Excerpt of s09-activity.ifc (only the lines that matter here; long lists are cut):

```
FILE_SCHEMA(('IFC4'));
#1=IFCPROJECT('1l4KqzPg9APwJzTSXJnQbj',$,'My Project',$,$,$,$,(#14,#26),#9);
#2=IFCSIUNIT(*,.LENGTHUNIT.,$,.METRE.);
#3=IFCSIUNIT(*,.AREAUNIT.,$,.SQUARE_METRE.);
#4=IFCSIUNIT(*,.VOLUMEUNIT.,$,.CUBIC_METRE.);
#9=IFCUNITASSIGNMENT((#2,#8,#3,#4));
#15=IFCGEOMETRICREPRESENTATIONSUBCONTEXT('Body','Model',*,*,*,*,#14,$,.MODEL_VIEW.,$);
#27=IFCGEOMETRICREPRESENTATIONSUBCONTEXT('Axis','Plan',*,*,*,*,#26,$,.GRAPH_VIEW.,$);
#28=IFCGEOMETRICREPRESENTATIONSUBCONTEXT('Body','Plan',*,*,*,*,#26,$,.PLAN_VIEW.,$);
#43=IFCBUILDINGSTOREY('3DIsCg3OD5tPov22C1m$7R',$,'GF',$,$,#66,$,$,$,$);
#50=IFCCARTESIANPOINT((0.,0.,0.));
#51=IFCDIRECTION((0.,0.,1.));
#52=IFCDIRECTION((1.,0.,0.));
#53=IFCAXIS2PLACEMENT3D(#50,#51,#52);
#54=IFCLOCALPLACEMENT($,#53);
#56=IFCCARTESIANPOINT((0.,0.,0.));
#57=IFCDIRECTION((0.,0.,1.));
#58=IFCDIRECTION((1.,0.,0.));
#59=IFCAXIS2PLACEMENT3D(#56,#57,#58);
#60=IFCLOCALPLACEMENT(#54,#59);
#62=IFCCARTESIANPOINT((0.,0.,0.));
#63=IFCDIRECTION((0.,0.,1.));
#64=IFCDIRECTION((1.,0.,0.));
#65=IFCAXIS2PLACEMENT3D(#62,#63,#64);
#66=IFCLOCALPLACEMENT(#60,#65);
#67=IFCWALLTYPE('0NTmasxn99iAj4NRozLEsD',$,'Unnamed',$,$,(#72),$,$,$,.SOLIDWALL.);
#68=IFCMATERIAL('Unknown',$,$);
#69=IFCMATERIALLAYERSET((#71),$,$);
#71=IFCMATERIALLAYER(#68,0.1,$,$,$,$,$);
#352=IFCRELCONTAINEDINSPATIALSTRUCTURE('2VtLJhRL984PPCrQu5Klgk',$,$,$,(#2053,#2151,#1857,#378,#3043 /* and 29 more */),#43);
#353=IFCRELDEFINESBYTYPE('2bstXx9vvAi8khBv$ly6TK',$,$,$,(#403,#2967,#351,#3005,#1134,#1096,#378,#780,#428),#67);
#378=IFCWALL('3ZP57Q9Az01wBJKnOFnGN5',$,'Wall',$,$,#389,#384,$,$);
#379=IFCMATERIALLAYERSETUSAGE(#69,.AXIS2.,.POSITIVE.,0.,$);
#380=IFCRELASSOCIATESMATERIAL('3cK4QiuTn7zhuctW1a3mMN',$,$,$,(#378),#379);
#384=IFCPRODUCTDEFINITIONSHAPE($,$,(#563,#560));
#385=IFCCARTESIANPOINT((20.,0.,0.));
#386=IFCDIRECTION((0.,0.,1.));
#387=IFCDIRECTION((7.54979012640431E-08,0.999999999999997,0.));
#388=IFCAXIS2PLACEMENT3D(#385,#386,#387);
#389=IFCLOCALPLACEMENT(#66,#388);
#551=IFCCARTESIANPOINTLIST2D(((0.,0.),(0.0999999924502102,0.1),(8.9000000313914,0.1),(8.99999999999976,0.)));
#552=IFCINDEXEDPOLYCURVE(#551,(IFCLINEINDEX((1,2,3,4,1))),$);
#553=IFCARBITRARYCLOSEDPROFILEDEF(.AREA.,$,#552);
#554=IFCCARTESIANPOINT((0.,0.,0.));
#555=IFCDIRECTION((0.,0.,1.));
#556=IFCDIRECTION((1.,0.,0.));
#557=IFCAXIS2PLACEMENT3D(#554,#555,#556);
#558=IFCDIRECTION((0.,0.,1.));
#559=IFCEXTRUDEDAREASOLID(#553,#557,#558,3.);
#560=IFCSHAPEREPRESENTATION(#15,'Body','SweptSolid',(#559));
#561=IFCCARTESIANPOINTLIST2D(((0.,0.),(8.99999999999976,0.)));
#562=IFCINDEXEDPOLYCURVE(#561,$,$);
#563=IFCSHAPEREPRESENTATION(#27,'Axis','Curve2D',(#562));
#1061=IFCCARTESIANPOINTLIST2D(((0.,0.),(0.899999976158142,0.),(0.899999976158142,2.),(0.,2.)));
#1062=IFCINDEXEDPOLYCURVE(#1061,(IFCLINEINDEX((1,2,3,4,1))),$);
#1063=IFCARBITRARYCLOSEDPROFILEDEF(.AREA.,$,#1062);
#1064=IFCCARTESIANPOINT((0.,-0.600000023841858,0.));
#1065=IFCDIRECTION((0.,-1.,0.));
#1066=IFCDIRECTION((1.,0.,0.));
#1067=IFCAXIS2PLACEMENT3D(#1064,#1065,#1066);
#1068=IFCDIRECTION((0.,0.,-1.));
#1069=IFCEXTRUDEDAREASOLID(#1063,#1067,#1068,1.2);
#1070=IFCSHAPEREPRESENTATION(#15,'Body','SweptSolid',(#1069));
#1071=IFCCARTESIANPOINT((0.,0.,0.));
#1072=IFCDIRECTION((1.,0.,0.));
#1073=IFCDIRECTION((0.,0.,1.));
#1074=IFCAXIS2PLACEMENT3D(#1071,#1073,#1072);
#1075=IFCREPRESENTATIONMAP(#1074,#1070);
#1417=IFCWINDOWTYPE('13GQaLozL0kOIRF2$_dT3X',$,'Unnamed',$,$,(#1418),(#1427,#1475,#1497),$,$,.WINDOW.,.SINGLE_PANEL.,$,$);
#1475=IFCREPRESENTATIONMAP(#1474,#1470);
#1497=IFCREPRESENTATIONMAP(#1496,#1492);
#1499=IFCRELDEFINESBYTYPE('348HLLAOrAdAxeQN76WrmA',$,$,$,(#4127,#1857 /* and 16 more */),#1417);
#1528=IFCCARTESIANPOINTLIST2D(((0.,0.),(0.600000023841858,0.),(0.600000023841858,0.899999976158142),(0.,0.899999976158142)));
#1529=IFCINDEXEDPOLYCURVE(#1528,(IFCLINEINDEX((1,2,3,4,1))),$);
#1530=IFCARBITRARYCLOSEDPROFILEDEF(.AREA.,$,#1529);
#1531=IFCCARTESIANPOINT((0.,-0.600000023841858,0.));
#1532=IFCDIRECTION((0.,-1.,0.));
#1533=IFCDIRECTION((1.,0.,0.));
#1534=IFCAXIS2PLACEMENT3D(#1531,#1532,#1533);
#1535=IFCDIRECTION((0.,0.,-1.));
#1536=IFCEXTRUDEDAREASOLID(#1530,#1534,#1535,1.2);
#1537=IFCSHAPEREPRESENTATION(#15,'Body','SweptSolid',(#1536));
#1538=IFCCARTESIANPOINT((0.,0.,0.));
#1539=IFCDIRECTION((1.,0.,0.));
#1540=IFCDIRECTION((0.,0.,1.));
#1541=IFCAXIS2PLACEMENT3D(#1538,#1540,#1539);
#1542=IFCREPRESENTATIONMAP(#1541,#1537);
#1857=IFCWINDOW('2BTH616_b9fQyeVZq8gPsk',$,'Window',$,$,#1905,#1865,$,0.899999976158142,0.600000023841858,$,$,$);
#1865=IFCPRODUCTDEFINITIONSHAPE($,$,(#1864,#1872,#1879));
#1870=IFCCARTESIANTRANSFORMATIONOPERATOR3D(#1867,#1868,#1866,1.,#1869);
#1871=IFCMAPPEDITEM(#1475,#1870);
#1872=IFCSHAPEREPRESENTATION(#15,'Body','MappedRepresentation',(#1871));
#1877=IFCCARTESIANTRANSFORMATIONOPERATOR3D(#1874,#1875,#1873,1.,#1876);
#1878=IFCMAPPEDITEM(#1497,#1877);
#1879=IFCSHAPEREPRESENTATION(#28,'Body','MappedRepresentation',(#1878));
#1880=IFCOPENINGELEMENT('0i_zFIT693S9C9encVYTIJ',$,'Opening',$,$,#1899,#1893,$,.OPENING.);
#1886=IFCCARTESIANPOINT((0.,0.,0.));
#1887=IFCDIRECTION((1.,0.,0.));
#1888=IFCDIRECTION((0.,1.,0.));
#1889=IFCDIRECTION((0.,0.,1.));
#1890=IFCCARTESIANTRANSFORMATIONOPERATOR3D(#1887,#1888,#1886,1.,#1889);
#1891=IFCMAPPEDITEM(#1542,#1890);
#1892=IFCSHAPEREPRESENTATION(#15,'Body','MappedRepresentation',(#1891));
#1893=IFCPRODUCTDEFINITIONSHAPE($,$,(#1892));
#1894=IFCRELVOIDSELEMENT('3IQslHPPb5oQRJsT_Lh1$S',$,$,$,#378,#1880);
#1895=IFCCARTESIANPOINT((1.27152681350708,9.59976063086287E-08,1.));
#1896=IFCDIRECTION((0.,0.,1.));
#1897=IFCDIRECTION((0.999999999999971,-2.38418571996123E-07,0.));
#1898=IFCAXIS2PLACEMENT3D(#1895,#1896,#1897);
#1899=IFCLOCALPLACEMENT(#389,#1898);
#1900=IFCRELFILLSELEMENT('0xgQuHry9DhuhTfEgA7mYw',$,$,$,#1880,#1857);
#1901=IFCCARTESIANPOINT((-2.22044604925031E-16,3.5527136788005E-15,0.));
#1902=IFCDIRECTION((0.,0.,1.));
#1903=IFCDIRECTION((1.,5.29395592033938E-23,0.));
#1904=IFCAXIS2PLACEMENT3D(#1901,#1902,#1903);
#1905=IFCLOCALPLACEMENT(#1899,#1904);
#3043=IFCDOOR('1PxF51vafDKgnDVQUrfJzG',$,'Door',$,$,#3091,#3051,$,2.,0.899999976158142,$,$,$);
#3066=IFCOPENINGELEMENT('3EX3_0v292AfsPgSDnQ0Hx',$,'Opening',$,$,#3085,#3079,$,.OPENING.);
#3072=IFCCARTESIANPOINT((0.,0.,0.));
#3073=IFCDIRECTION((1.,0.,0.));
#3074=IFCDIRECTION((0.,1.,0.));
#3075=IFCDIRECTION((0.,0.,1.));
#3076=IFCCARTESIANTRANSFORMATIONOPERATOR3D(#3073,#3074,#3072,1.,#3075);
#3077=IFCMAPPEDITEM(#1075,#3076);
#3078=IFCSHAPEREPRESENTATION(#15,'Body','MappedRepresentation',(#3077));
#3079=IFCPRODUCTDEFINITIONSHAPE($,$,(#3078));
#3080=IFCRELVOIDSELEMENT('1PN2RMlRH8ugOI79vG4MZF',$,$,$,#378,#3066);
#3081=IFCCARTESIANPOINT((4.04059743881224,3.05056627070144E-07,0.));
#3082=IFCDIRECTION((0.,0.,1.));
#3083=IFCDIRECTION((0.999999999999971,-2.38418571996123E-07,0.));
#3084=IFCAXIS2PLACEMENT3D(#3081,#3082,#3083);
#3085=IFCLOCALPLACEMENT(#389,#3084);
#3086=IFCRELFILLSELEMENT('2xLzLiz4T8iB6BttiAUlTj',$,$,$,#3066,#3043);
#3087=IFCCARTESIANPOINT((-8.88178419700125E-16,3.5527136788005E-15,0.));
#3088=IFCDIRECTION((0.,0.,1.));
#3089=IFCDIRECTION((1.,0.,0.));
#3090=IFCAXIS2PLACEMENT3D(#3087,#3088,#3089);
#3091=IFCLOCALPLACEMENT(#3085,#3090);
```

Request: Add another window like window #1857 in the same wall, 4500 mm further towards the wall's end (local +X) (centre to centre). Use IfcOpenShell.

```python
import ifcopenshell
import ifcopenshell.api.feature
import ifcopenshell.api.geometry
import ifcopenshell.api.root
import ifcopenshell.geom
import ifcopenshell.util.element
import ifcopenshell.util.placement
import ifcopenshell.util.shape
import ifcopenshell.util.unit

model = ifcopenshell.open("s09-activity.ifc")
unit_scale = ifcopenshell.util.unit.calculate_unit_scale(model)
settings = ifcopenshell.geom.settings()


def volume(element):
    """Net volume in cubic metres, openings subtracted."""
    shape = ifcopenshell.geom.create_shape(settings, element)
    return ifcopenshell.util.shape.get_volume(shape.geometry)


window = model.by_guid("2BTH616_b9fQyeVZq8gPsk")
opening = window.FillsVoids[0].RelatingOpeningElement
wall = opening.VoidsElements[0].RelatingBuildingElement
before = volume(wall)
shift = ifcopenshell.util.placement.get_local_placement(wall.ObjectPlacement)[:3, 0] * 4.5 / unit_scale

# copy_class copies the void relationship, type, container and properties, but no geometry.
new_opening = ifcopenshell.api.root.copy_class(model, product=opening)
new_opening.Representation = ifcopenshell.util.element.copy_deep(
    model, opening.Representation, exclude=["IfcGeometricRepresentationContext", "IfcRepresentationMap"]
)
new_window = ifcopenshell.api.root.copy_class(model, product=window)
new_window.Representation = ifcopenshell.util.element.copy_deep(
    model, window.Representation, exclude=["IfcGeometricRepresentationContext", "IfcRepresentationMap"]
)
ifcopenshell.api.feature.add_filling(model, opening=new_opening, element=new_window)

for old, new in ((opening, new_opening), (window, new_window)):
    matrix = ifcopenshell.util.placement.get_local_placement(old.ObjectPlacement)
    matrix[:3, 3] += shift
    ifcopenshell.api.geometry.edit_object_placement(model, product=new, matrix=matrix, is_si=False)

after = volume(wall)

print(f"wall volume {before:.3f} -> {after:.3f} m3")

model.write("s09-activity_updated.ifc")
```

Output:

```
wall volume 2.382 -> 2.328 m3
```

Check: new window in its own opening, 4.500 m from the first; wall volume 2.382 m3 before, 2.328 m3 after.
